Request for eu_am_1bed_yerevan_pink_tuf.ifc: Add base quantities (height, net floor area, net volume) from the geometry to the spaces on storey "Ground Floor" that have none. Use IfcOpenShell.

First a look at what the model holds.

```python
import ifcopenshell
import ifcopenshell.util.element
import ifcopenshell.util.unit

model = ifcopenshell.open("eu_am_1bed_yerevan_pink_tuf.ifc")
print(model.schema)
for unit_type in ("LENGTHUNIT", "AREAUNIT", "VOLUMEUNIT"):
    print(unit_type, ifcopenshell.util.unit.calculate_unit_scale(model, unit_type))
storey = next(s for s in model.by_type("IfcBuildingStorey") if s.Name == "Ground Floor")
spaces = [e for e in ifcopenshell.util.element.get_decomposition(storey) if e.is_a("IfcSpace")]
for e in sorted(spaces, key=lambda e: e.id()):
    print(e.id(), e.is_a(), e.Name, list(ifcopenshell.util.element.get_psets(e, qtos_only=True)), sep=" | ")
```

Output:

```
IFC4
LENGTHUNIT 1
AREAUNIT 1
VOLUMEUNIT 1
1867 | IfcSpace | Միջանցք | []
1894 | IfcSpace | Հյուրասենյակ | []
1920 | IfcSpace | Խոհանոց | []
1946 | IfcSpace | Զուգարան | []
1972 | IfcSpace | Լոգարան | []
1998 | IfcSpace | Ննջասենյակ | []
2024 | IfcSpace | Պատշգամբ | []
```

```python
import ifcopenshell
import ifcopenshell.api.pset
import ifcopenshell.geom
import ifcopenshell.util.element
import ifcopenshell.util.shape
import ifcopenshell.util.unit

model = ifcopenshell.open("eu_am_1bed_yerevan_pink_tuf.ifc")
unit_scale = ifcopenshell.util.unit.calculate_unit_scale(model)
area_scale = ifcopenshell.util.unit.calculate_unit_scale(model, "AREAUNIT")
volume_scale = ifcopenshell.util.unit.calculate_unit_scale(model, "VOLUMEUNIT")
settings = ifcopenshell.geom.settings()

storey = next(s for s in model.by_type("IfcBuildingStorey") if s.Name == "Ground Floor")
spaces = [e for e in ifcopenshell.util.element.get_decomposition(storey) if e.is_a("IfcSpace")]

for e in sorted(spaces, key=lambda e: e.id()):
    if ifcopenshell.util.element.get_psets(e, qtos_only=True, should_inherit=False):
        continue
    # Geometry comes back in metres, in the element's own axes.
    shape = ifcopenshell.geom.create_shape(settings, e)
    values = {
        "Height": ifcopenshell.util.shape.get_z(shape.geometry) / unit_scale,
        "NetFloorArea": ifcopenshell.util.shape.get_footprint_area(shape.geometry) / area_scale,
        "NetVolume": ifcopenshell.util.shape.get_volume(shape.geometry) / volume_scale,
    }
    qto = ifcopenshell.api.pset.add_qto(model, product=e, name="Qto_SpaceBaseQuantities")
    ifcopenshell.api.pset.edit_qto(model, qto=qto, properties=values)
    print(e.id(), {k: round(v, 3) for k, v in values.items()})

model.write("eu_am_1bed_yerevan_pink_tuf_edited.ifc")
```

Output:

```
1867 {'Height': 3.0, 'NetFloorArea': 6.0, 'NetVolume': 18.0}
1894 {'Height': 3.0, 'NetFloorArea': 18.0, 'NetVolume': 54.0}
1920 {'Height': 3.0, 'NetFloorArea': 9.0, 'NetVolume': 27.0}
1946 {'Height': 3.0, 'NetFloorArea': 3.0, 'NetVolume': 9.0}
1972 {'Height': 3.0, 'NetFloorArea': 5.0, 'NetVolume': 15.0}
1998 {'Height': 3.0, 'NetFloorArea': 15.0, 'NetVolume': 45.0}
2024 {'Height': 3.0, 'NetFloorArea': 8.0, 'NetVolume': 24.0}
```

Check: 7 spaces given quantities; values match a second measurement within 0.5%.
